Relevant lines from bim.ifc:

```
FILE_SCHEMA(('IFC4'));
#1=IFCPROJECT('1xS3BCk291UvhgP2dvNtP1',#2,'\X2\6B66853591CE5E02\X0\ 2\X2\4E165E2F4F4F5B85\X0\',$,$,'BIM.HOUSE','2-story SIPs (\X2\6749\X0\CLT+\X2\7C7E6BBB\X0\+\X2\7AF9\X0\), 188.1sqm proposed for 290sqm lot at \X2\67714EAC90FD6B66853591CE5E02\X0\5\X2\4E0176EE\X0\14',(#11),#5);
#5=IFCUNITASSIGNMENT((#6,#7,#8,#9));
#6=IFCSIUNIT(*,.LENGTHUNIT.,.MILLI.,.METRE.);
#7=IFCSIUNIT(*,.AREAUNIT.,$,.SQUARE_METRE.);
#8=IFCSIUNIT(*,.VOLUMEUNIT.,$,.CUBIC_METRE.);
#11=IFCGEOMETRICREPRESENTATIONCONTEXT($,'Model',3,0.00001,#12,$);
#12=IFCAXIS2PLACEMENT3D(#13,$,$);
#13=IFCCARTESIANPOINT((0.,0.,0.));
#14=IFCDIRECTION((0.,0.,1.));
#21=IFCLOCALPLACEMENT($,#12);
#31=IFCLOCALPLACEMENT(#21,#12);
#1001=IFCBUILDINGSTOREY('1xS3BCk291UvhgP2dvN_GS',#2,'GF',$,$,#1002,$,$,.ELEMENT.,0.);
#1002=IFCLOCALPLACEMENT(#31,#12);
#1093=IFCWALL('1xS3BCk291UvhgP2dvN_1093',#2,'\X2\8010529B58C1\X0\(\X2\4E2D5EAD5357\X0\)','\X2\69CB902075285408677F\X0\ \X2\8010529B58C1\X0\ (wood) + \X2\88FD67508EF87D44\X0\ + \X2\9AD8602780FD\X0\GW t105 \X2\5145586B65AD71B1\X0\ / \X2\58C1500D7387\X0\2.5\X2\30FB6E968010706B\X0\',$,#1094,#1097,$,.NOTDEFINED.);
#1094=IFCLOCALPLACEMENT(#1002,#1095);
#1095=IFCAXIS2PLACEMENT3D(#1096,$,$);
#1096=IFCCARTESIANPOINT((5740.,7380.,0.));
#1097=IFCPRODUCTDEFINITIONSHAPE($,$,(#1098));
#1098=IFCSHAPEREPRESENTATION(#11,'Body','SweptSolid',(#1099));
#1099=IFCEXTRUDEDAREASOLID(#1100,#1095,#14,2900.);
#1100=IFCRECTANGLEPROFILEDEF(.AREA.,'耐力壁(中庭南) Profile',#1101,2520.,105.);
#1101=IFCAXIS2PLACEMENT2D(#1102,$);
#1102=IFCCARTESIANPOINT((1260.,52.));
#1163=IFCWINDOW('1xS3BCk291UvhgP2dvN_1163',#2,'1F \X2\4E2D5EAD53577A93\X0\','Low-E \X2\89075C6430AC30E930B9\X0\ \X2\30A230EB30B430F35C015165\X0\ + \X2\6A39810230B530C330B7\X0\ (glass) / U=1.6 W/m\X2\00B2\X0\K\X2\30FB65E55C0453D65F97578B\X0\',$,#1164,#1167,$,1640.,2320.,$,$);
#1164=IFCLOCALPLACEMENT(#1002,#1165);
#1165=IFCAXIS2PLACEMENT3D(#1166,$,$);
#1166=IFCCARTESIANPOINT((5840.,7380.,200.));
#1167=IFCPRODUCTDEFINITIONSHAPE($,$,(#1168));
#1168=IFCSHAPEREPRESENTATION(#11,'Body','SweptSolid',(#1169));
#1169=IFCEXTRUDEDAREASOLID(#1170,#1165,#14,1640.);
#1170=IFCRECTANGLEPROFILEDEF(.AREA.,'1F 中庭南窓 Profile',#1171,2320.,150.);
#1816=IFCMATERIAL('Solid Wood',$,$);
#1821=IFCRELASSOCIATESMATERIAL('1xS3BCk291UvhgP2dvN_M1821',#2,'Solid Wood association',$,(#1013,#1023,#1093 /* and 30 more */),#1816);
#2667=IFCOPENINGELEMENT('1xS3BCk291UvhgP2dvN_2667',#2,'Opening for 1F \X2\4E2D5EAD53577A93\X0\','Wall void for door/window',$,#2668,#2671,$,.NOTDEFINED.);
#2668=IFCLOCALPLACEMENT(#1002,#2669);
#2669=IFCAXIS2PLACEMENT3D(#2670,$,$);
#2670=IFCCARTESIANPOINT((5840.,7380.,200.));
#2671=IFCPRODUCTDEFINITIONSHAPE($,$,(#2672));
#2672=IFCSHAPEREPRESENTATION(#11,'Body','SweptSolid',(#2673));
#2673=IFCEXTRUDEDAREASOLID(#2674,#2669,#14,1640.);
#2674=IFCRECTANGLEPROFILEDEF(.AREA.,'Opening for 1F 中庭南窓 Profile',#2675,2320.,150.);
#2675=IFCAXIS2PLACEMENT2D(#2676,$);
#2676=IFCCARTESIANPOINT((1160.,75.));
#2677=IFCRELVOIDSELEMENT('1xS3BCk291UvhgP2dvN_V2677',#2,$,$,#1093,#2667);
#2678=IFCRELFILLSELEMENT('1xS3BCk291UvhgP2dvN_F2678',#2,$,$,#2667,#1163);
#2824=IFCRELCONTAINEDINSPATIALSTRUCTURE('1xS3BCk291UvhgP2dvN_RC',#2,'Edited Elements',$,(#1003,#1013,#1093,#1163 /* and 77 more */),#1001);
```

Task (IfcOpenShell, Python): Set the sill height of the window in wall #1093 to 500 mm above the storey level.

```python
import numpy as np
import ifcopenshell
import ifcopenshell.api.geometry
import ifcopenshell.geom
import ifcopenshell.util.element
import ifcopenshell.util.placement
import ifcopenshell.util.shape
import ifcopenshell.util.unit

model = ifcopenshell.open("bim.ifc")
unit_scale = ifcopenshell.util.unit.calculate_unit_scale(model)

window = model.by_guid("1xS3BCk291UvhgP2dvN_1163")
opening = window.FillsVoids[0].RelatingOpeningElement
storey = ifcopenshell.util.element.get_container(window, ifc_class="IfcBuildingStorey")
level = ifcopenshell.util.placement.get_local_placement(storey.ObjectPlacement)[2, 3]

# The opening's origin need not be at the sill, so measure its lowest point.
shape = ifcopenshell.geom.create_shape(ifcopenshell.geom.settings(), opening)
bottom = ifcopenshell.util.shape.get_shape_bottom_elevation(shape, shape.geometry) / unit_scale
dz = level + 0.5 / unit_scale - bottom

shift = np.array([0.0, 0.0, dz])
# The window is not placed relative to its opening, so move both.
for product in (opening, window):
    matrix = ifcopenshell.util.placement.get_local_placement(product.ObjectPlacement)
    matrix[:3, 3] += shift
    ifcopenshell.api.geometry.edit_object_placement(model, product=product, matrix=matrix, is_si=False)

print(f"moved by {dz * unit_scale:+.3f} m")

model.write("bim_edited.ifc")
```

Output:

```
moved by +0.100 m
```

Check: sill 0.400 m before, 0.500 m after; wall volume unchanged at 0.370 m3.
